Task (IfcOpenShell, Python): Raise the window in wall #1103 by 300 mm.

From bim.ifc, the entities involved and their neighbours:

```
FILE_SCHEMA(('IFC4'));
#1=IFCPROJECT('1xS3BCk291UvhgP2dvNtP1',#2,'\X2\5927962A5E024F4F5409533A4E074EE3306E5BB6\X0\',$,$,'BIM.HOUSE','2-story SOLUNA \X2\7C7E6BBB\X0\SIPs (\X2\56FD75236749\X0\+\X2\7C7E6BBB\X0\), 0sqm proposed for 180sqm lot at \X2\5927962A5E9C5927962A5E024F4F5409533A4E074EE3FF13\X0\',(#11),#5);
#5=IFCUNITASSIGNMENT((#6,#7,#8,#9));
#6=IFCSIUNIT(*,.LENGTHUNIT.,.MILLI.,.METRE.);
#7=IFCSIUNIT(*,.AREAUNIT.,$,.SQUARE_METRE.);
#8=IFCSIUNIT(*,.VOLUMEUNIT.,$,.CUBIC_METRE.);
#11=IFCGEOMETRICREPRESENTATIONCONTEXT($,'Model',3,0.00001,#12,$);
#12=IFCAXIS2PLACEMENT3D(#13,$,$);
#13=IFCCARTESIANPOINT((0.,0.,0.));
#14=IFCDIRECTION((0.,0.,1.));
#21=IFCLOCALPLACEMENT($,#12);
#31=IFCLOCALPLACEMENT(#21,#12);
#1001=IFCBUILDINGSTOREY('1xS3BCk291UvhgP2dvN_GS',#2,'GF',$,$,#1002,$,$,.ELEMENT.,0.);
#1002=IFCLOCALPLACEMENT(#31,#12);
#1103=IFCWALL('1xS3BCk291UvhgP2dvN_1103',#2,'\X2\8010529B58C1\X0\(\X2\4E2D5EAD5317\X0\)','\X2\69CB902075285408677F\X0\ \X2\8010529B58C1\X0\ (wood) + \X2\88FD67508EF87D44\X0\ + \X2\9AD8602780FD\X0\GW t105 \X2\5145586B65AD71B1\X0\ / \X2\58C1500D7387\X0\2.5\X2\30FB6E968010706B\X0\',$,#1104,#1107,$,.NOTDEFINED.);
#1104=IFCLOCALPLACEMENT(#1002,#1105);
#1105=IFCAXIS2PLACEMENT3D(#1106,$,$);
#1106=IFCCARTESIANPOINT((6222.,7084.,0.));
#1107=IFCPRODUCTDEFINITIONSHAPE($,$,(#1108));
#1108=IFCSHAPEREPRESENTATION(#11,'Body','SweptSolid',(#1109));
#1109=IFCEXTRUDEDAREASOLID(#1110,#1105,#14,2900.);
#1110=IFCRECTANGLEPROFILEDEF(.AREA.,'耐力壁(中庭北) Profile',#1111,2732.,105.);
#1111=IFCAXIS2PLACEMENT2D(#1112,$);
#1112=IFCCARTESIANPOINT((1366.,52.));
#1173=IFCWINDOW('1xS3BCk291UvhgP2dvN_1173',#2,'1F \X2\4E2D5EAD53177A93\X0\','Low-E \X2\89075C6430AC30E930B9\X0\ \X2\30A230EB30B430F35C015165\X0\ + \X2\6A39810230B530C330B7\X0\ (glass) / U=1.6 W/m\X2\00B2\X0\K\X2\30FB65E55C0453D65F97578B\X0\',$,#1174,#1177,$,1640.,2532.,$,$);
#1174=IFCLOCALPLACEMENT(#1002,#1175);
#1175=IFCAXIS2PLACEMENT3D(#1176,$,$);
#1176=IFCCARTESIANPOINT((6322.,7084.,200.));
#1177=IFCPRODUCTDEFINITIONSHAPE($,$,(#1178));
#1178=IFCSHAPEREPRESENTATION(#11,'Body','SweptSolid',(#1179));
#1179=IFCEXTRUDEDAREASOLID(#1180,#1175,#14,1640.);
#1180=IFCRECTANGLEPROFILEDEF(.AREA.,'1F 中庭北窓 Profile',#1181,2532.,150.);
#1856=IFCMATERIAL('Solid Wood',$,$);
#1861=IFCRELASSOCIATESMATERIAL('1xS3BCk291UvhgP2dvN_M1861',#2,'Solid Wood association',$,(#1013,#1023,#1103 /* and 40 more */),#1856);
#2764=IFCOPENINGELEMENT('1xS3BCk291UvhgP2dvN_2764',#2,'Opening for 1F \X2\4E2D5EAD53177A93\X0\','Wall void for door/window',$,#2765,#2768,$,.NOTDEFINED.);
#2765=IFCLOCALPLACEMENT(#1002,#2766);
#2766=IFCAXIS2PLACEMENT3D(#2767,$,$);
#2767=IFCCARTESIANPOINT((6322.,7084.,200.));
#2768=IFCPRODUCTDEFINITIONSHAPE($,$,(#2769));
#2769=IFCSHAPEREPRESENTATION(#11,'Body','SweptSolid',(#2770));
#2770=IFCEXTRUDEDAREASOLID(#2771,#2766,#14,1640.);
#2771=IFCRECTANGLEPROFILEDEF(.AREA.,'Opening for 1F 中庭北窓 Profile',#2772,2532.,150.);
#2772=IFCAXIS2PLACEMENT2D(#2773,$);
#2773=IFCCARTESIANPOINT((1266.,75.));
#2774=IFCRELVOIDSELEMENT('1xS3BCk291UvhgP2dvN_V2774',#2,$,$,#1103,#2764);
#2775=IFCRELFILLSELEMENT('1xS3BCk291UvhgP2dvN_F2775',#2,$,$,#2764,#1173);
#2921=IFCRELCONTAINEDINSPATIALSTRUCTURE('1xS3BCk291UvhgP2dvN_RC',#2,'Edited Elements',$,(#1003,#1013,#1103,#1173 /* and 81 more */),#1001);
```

```python
import numpy as np
import ifcopenshell
import ifcopenshell.api.geometry
import ifcopenshell.util.placement
import ifcopenshell.util.unit

model = ifcopenshell.open("bim.ifc")
unit_scale = ifcopenshell.util.unit.calculate_unit_scale(model)

window = model.by_id(1173)
opening = window.FillsVoids[0].RelatingOpeningElement
dz = 0.3 / unit_scale

shift = np.array([0.0, 0.0, dz])
# The window is not placed relative to its opening, so move both.
for product in (opening, window):
    matrix = ifcopenshell.util.placement.get_local_placement(product.ObjectPlacement)
    matrix[:3, 3] += shift
    ifcopenshell.api.geometry.edit_object_placement(model, product=product, matrix=matrix, is_si=False)

print(f"moved by {dz * unit_scale:+.3f} m")

model.write("bim-out.ifc")
```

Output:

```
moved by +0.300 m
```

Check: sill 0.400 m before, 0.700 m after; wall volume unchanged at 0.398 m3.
